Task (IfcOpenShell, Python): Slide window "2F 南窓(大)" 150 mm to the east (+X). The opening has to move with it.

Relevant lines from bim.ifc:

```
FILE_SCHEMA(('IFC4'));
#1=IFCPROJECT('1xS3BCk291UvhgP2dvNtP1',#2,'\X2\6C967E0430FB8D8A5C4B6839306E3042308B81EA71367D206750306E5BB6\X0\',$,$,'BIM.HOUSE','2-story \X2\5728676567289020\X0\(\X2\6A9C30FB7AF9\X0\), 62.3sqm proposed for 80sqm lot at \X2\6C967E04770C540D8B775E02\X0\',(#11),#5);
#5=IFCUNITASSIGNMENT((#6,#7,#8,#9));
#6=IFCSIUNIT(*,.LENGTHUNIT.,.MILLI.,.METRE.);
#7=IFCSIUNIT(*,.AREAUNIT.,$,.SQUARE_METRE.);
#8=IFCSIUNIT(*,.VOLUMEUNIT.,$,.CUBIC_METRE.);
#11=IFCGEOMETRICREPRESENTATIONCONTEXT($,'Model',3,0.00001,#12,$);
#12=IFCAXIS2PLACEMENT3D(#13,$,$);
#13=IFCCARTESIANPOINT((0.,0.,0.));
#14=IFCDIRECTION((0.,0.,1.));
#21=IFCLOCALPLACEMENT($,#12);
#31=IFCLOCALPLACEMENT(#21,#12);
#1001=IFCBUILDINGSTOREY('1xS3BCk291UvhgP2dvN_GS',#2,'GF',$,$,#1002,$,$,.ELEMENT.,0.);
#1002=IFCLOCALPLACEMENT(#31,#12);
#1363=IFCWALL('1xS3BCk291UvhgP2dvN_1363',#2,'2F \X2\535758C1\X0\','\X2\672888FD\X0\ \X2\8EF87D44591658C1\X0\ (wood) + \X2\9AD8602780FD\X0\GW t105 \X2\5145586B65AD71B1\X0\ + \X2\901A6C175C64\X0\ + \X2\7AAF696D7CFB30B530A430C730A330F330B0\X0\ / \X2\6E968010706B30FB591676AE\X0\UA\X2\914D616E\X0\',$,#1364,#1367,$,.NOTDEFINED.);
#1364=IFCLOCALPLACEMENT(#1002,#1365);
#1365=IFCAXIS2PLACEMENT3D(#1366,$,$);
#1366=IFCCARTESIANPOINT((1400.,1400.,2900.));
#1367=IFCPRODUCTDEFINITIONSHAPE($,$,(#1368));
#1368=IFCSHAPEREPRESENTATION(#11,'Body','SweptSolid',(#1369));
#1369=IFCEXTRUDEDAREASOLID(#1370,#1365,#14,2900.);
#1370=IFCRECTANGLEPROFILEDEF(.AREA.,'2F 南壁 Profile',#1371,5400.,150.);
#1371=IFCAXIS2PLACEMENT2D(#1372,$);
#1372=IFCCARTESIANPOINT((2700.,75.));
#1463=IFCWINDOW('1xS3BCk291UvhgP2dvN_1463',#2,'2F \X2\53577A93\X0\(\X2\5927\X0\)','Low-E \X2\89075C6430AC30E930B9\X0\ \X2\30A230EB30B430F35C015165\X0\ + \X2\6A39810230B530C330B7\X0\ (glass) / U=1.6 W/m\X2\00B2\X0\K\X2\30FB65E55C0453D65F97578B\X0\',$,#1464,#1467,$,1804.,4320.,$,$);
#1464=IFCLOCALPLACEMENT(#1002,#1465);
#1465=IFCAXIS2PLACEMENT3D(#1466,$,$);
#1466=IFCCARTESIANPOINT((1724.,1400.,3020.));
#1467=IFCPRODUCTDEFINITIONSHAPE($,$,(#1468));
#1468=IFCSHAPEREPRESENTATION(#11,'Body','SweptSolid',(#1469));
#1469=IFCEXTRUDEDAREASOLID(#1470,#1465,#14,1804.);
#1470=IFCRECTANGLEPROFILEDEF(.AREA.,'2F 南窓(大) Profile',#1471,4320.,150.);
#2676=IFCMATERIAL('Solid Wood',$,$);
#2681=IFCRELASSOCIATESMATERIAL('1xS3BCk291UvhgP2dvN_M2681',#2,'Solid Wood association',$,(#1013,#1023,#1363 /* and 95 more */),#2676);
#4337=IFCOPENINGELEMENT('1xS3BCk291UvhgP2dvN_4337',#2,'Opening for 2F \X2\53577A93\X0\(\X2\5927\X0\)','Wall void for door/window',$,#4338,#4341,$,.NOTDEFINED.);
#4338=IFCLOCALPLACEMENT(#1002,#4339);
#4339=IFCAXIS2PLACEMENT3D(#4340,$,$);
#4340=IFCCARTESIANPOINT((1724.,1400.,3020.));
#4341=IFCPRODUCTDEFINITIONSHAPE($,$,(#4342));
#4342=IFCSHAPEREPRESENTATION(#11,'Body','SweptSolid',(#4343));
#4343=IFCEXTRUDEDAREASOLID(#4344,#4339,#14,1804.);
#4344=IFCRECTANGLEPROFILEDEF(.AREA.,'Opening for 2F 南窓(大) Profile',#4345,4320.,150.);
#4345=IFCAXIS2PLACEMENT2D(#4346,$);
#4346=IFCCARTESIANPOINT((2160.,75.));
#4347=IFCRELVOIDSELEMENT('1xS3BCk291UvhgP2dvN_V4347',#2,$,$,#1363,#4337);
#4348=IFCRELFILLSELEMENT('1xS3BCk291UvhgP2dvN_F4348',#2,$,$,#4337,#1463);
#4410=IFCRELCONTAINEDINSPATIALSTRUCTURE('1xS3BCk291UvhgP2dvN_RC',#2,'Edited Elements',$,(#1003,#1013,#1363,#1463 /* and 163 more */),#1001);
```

```python
import ifcopenshell
import ifcopenshell.api.geometry
import ifcopenshell.util.placement

model = ifcopenshell.open("bim.ifc")

window = model.by_id(1463)
opening = window.FillsVoids[0].RelatingOpeningElement
wall = opening.VoidsElements[0].RelatingBuildingElement

wall_matrix = ifcopenshell.util.placement.get_local_placement(wall.ObjectPlacement)
shift = wall_matrix[:3, 0] * 150.0
before = ifcopenshell.util.placement.get_local_placement(window.ObjectPlacement)[:3, 3].copy()

# The window is not placed relative to its opening, so move both.
for product in (opening, window):
    matrix = ifcopenshell.util.placement.get_local_placement(product.ObjectPlacement)
    matrix[:3, 3] += shift
    ifcopenshell.api.geometry.edit_object_placement(model, product=product, matrix=matrix, is_si=False)

after = ifcopenshell.util.placement.get_local_placement(window.ObjectPlacement)[:3, 3]
print("window moved by", (after - before).round(3) + 0.0)

model.write("bim_v2.ifc")
```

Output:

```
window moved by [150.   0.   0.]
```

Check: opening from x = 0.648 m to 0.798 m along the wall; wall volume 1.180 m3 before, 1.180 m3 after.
